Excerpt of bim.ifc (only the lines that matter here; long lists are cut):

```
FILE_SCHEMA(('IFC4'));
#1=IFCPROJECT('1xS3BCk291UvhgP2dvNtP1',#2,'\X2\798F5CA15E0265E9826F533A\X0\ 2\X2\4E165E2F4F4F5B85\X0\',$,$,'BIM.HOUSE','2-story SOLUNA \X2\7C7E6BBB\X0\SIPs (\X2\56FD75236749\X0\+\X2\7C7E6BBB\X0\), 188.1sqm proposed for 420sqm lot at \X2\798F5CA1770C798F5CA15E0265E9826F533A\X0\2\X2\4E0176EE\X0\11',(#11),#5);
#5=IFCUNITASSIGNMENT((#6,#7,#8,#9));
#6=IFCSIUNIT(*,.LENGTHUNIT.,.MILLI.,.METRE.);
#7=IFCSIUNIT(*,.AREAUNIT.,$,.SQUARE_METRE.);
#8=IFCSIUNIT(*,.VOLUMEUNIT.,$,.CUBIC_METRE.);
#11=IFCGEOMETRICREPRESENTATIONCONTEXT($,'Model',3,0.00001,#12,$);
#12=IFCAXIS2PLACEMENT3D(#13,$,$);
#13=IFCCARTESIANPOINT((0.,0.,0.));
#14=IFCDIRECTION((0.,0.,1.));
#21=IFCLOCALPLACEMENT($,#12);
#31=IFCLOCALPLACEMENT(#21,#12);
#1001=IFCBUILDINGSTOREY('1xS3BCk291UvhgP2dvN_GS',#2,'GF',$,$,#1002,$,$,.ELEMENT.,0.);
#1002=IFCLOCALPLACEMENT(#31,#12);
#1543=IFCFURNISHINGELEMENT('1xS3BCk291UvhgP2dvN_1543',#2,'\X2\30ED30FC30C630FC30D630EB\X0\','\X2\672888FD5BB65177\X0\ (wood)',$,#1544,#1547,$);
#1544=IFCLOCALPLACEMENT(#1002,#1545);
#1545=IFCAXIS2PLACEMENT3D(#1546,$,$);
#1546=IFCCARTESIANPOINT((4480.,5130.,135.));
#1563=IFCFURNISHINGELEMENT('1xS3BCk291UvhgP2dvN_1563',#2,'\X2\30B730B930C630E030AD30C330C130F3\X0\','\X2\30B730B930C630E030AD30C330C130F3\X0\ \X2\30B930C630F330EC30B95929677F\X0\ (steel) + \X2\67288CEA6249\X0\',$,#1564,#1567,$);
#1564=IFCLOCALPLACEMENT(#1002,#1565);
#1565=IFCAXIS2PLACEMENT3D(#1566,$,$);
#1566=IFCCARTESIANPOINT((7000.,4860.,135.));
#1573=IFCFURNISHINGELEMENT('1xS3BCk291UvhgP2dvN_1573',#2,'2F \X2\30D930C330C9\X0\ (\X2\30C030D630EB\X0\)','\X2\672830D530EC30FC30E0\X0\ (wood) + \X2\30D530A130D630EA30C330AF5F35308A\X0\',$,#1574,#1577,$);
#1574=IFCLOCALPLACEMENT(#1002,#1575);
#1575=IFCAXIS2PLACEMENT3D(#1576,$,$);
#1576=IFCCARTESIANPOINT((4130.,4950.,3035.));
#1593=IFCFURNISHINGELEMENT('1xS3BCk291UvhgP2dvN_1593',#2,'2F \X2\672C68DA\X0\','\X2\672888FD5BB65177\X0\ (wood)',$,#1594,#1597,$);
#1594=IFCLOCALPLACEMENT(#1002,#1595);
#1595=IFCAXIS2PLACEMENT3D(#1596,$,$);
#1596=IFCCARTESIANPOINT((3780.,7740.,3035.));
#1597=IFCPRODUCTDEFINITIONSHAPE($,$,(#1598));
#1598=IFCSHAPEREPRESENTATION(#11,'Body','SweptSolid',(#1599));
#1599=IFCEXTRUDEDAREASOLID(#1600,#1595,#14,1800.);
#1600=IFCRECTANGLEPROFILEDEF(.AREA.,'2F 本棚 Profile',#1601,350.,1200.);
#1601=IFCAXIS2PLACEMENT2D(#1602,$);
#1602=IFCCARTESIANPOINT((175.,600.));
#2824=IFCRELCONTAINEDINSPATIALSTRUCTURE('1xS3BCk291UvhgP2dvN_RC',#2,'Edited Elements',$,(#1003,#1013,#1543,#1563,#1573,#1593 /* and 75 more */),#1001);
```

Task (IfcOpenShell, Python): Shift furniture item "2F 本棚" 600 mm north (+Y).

```python
import ifcopenshell
import ifcopenshell.api.geometry
import ifcopenshell.util.placement

model = ifcopenshell.open("bim.ifc")

item = model.by_guid("1xS3BCk291UvhgP2dvN_1593")
matrix = ifcopenshell.util.placement.get_local_placement(item.ObjectPlacement)
matrix[1, 3] += 600.0
ifcopenshell.api.geometry.edit_object_placement(model, product=item, matrix=matrix, is_si=False)

print(ifcopenshell.util.placement.get_local_placement(item.ObjectPlacement).round(3) + 0.0)

model.write("bim_rev.ifc")
```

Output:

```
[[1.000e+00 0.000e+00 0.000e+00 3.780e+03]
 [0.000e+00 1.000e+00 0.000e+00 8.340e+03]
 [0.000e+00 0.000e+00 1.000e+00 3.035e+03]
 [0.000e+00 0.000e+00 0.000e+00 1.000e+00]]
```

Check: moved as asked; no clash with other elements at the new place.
